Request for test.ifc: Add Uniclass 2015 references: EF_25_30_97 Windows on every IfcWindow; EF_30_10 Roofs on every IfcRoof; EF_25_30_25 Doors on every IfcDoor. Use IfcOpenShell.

First a look at what the model holds.

```python
import ifcopenshell

model = ifcopenshell.open("test.ifc")
print(model.schema)
print("classifications:", [c.Name for c in model.by_type("IfcClassification")])
for ifc_class in ("IfcDoor", "IfcRoof", "IfcStair", "IfcWall", "IfcWindow"):
    print(ifc_class, len(model.by_type(ifc_class)))
```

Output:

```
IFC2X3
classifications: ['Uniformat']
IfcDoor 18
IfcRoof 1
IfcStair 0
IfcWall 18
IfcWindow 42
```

```python
import ifcopenshell
import ifcopenshell.api.classification

model = ifcopenshell.open("test.ifc")

# IFC2X3 requires Source and Edition and has no link from the project to the system.
system = model.create_entity("IfcClassification", Source="NBS", Edition="2015", Name="Uniclass 2015")

codes = {
    "IfcWindow": ("EF_25_30_97", "Windows"),
    "IfcRoof": ("EF_30_10", "Roofs"),
    "IfcDoor": ("EF_25_30_25", "Doors"),
}
for ifc_class, (code, name) in codes.items():
    products = model.by_type(ifc_class)
    ifcopenshell.api.classification.add_reference(
        model, products=products, classification=system, identification=code, name=name
    )
    print(code, len(products))

model.write("test_v2.ifc")
```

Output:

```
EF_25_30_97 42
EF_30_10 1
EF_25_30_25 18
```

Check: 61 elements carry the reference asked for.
